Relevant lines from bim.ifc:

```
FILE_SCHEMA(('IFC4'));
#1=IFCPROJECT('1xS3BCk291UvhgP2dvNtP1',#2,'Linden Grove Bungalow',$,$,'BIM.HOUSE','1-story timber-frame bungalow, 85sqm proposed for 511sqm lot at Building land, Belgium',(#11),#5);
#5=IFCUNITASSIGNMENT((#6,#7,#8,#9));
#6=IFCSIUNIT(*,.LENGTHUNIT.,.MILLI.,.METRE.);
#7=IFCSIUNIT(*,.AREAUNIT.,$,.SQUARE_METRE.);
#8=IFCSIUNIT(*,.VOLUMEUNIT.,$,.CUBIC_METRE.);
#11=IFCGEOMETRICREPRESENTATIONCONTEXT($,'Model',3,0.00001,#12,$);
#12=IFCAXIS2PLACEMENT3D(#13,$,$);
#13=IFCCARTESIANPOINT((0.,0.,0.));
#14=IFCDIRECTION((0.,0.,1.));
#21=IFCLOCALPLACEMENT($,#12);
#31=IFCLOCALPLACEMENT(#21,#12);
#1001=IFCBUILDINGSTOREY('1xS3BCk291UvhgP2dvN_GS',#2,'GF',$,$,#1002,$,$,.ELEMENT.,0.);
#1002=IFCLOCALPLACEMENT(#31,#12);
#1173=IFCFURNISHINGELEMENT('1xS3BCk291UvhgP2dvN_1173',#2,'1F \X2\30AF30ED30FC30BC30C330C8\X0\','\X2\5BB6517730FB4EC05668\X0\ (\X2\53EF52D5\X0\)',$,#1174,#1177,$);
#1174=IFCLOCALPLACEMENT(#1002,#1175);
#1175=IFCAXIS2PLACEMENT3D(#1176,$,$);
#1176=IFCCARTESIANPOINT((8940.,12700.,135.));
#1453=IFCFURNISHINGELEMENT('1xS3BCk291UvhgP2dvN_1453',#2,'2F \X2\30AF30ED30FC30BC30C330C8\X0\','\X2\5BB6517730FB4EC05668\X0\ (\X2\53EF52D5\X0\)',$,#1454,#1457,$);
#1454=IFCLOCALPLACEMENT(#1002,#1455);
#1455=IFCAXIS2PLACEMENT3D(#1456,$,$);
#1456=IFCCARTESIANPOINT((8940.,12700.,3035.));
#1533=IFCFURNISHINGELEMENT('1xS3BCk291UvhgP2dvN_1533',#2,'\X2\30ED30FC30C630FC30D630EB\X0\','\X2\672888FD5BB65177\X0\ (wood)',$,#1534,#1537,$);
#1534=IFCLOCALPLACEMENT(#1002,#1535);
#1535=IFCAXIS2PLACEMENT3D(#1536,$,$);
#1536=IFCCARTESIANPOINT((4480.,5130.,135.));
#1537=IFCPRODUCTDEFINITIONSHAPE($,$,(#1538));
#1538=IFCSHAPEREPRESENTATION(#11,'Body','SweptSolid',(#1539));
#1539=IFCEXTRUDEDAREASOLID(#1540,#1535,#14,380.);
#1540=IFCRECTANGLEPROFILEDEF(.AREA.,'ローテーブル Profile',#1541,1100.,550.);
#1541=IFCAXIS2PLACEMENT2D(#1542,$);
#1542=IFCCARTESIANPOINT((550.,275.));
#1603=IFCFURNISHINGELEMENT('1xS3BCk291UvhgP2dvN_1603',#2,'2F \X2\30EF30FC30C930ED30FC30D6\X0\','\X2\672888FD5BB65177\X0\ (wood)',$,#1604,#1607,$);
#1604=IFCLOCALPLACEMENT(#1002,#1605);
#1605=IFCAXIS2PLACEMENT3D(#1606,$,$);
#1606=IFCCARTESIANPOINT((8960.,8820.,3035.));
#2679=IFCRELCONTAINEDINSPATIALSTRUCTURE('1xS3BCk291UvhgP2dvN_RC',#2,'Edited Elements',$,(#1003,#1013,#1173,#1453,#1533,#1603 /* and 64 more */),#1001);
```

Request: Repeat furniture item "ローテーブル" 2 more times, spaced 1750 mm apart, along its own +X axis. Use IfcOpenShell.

```python
import ifcopenshell
import ifcopenshell.api.geometry
import ifcopenshell.api.root
import ifcopenshell.util.element
import ifcopenshell.util.placement

model = ifcopenshell.open("bim.ifc")


def reuse_history(source, copy):
    """copy_class also copies each property set's owner history, people and application; keep the originals."""
    for rel in copy.IsDefinedBy:
        if rel.is_a("IfcRelDefinesByProperties") and (history := rel.RelatingPropertyDefinition.OwnerHistory):
            rel.RelatingPropertyDefinition.OwnerHistory = source.OwnerHistory
            ifcopenshell.util.element.remove_deep2(model, history)


source = model.by_guid("1xS3BCk291UvhgP2dvN_1533")
base = ifcopenshell.util.placement.get_local_placement(source.ObjectPlacement)
step = base[:3, 0] * 1750.0

for i in range(1, 3):
    copy = ifcopenshell.api.root.copy_class(model, product=source)
    copy.Representation = ifcopenshell.util.element.copy_deep(
        model, source.Representation, exclude=["IfcGeometricRepresentationContext", "IfcRepresentationMap"]
    )
    reuse_history(source, copy)
    matrix = base.copy()
    matrix[:3, 3] += i * step
    print("added at", matrix[:3, 3].round(3) + 0.0)
    ifcopenshell.api.geometry.edit_object_placement(model, product=copy, matrix=matrix, is_si=False)

model.write("bim_rev.ifc")
```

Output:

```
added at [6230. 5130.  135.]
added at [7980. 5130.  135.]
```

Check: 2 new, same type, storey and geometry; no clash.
